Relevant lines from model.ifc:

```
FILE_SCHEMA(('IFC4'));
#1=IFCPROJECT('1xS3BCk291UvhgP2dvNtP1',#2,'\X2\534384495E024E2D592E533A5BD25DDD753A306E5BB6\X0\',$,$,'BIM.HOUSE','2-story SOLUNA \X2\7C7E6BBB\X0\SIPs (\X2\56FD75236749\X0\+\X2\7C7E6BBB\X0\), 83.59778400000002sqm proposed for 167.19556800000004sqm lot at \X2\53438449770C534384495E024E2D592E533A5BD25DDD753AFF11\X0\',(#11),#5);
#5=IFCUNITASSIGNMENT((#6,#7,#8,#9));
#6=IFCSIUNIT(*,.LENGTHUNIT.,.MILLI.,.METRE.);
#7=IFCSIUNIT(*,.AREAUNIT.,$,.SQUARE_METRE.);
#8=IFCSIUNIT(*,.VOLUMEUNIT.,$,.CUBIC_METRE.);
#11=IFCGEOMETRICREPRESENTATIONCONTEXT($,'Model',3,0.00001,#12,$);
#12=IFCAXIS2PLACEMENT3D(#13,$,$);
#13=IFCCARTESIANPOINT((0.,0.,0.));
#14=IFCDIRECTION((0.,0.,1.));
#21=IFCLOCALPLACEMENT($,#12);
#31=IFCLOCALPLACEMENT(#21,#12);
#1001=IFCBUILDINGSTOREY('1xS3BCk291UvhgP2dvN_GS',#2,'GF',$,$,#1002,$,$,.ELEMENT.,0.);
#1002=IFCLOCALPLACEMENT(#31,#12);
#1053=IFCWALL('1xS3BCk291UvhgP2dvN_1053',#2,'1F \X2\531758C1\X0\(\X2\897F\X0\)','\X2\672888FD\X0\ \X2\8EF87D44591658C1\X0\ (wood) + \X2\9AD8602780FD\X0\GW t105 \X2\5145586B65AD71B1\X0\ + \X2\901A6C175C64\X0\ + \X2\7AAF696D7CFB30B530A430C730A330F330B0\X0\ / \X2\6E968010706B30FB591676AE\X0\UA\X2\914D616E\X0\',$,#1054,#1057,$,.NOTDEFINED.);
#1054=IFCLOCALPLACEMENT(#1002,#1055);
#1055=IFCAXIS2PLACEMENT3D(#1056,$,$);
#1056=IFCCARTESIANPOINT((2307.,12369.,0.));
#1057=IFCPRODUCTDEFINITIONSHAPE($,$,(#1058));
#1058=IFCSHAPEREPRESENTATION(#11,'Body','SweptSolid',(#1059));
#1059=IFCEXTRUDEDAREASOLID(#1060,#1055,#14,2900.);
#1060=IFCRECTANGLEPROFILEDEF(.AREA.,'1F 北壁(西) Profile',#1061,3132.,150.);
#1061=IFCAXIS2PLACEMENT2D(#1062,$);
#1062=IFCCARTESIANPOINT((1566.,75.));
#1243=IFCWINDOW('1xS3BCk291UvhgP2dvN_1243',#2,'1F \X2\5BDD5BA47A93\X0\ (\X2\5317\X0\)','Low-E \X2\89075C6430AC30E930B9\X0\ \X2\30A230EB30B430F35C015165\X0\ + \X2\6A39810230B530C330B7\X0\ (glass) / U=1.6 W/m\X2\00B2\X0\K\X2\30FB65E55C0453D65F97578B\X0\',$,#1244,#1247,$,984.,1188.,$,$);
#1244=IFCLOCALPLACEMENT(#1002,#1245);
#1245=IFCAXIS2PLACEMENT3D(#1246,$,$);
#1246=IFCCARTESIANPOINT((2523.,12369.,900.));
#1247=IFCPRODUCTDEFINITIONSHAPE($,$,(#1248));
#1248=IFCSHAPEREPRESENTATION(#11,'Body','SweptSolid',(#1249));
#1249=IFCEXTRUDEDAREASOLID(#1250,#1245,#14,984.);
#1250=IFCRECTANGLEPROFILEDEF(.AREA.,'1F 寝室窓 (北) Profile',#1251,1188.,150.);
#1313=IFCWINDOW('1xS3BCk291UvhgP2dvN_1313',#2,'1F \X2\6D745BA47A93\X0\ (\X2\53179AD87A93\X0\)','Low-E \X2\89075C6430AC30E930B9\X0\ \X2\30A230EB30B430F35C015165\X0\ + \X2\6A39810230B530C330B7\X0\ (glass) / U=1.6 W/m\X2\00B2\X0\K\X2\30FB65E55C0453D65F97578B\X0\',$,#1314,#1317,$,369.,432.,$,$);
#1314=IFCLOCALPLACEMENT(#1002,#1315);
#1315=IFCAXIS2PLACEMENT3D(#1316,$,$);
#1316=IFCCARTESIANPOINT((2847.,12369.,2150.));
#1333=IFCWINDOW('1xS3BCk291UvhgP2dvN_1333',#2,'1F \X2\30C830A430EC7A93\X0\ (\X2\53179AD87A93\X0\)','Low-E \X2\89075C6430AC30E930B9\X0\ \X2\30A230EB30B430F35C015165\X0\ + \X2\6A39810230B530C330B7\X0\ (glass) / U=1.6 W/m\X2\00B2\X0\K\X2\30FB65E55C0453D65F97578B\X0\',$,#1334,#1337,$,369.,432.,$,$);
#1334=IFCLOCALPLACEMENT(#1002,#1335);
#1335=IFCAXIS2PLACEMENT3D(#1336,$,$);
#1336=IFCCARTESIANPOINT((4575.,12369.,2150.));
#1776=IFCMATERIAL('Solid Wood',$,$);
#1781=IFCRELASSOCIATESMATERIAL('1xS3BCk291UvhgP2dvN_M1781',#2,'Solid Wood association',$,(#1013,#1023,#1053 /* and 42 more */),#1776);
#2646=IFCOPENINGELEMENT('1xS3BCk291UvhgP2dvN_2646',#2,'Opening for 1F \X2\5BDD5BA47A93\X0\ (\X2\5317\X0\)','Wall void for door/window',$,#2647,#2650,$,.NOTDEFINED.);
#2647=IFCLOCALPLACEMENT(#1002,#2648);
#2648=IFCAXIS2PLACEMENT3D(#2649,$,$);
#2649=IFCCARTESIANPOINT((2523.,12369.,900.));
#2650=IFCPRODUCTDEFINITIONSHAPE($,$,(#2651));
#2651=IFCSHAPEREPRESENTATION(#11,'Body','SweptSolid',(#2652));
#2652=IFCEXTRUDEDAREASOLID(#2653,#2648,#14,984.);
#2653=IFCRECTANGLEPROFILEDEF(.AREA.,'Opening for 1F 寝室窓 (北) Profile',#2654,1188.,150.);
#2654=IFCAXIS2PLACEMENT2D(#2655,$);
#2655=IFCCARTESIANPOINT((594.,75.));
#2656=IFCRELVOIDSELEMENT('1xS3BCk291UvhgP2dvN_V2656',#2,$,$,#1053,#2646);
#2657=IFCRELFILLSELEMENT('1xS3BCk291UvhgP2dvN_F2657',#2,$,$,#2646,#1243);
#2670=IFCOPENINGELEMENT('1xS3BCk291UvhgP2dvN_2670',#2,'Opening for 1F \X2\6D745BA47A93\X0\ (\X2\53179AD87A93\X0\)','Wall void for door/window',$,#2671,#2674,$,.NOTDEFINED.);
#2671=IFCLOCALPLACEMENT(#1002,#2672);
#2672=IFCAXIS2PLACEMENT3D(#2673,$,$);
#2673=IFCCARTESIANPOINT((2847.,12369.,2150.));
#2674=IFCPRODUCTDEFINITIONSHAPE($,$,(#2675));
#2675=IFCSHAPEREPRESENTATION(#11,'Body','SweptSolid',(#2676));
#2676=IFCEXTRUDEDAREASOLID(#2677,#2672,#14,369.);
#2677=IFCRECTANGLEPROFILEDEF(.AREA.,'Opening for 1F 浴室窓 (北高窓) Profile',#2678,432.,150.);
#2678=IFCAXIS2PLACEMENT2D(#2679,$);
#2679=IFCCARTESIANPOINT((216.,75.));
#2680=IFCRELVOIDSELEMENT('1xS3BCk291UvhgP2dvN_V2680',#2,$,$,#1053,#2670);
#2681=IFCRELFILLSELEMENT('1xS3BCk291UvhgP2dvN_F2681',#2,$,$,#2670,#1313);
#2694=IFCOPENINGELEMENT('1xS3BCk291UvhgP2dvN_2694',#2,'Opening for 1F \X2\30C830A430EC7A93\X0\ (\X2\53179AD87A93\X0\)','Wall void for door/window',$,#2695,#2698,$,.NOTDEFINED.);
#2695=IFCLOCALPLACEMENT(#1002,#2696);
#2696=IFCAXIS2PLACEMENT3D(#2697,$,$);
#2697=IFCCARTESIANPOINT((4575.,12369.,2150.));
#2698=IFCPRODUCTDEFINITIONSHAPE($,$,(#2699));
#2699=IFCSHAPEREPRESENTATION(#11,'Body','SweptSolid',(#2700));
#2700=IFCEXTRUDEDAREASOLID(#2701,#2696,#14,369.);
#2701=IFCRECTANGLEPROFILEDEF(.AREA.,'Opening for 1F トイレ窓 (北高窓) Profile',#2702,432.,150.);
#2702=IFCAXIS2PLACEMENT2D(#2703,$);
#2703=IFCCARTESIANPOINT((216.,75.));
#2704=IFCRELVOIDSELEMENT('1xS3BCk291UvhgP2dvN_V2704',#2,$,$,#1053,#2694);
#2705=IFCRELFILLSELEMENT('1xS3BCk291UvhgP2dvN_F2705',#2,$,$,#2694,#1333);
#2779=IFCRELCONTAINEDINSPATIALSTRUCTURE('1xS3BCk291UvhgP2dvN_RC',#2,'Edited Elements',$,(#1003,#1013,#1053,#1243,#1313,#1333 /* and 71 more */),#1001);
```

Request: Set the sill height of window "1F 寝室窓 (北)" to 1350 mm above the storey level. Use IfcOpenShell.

```python
import numpy as np
import ifcopenshell
import ifcopenshell.api.geometry
import ifcopenshell.geom
import ifcopenshell.util.element
import ifcopenshell.util.placement
import ifcopenshell.util.shape
import ifcopenshell.util.unit

model = ifcopenshell.open("model.ifc")
unit_scale = ifcopenshell.util.unit.calculate_unit_scale(model)

window = model.by_id(1243)
opening = window.FillsVoids[0].RelatingOpeningElement
storey = ifcopenshell.util.element.get_container(window, ifc_class="IfcBuildingStorey")
level = ifcopenshell.util.placement.get_local_placement(storey.ObjectPlacement)[2, 3]

# The opening's origin need not be at the sill, so measure its lowest point.
shape = ifcopenshell.geom.create_shape(ifcopenshell.geom.settings(), opening)
bottom = ifcopenshell.util.shape.get_shape_bottom_elevation(shape, shape.geometry) / unit_scale
dz = level + 1.35 / unit_scale - bottom

shift = np.array([0.0, 0.0, dz])
# The window is not placed relative to its opening, so move both.
for product in (opening, window):
    matrix = ifcopenshell.util.placement.get_local_placement(product.ObjectPlacement)
    matrix[:3, 3] += shift
    ifcopenshell.api.geometry.edit_object_placement(model, product=product, matrix=matrix, is_si=False)

print(f"moved by {dz * unit_scale:+.3f} m")

model.write("model-out.ifc")
```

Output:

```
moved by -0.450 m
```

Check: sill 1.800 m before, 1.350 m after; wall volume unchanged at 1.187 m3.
